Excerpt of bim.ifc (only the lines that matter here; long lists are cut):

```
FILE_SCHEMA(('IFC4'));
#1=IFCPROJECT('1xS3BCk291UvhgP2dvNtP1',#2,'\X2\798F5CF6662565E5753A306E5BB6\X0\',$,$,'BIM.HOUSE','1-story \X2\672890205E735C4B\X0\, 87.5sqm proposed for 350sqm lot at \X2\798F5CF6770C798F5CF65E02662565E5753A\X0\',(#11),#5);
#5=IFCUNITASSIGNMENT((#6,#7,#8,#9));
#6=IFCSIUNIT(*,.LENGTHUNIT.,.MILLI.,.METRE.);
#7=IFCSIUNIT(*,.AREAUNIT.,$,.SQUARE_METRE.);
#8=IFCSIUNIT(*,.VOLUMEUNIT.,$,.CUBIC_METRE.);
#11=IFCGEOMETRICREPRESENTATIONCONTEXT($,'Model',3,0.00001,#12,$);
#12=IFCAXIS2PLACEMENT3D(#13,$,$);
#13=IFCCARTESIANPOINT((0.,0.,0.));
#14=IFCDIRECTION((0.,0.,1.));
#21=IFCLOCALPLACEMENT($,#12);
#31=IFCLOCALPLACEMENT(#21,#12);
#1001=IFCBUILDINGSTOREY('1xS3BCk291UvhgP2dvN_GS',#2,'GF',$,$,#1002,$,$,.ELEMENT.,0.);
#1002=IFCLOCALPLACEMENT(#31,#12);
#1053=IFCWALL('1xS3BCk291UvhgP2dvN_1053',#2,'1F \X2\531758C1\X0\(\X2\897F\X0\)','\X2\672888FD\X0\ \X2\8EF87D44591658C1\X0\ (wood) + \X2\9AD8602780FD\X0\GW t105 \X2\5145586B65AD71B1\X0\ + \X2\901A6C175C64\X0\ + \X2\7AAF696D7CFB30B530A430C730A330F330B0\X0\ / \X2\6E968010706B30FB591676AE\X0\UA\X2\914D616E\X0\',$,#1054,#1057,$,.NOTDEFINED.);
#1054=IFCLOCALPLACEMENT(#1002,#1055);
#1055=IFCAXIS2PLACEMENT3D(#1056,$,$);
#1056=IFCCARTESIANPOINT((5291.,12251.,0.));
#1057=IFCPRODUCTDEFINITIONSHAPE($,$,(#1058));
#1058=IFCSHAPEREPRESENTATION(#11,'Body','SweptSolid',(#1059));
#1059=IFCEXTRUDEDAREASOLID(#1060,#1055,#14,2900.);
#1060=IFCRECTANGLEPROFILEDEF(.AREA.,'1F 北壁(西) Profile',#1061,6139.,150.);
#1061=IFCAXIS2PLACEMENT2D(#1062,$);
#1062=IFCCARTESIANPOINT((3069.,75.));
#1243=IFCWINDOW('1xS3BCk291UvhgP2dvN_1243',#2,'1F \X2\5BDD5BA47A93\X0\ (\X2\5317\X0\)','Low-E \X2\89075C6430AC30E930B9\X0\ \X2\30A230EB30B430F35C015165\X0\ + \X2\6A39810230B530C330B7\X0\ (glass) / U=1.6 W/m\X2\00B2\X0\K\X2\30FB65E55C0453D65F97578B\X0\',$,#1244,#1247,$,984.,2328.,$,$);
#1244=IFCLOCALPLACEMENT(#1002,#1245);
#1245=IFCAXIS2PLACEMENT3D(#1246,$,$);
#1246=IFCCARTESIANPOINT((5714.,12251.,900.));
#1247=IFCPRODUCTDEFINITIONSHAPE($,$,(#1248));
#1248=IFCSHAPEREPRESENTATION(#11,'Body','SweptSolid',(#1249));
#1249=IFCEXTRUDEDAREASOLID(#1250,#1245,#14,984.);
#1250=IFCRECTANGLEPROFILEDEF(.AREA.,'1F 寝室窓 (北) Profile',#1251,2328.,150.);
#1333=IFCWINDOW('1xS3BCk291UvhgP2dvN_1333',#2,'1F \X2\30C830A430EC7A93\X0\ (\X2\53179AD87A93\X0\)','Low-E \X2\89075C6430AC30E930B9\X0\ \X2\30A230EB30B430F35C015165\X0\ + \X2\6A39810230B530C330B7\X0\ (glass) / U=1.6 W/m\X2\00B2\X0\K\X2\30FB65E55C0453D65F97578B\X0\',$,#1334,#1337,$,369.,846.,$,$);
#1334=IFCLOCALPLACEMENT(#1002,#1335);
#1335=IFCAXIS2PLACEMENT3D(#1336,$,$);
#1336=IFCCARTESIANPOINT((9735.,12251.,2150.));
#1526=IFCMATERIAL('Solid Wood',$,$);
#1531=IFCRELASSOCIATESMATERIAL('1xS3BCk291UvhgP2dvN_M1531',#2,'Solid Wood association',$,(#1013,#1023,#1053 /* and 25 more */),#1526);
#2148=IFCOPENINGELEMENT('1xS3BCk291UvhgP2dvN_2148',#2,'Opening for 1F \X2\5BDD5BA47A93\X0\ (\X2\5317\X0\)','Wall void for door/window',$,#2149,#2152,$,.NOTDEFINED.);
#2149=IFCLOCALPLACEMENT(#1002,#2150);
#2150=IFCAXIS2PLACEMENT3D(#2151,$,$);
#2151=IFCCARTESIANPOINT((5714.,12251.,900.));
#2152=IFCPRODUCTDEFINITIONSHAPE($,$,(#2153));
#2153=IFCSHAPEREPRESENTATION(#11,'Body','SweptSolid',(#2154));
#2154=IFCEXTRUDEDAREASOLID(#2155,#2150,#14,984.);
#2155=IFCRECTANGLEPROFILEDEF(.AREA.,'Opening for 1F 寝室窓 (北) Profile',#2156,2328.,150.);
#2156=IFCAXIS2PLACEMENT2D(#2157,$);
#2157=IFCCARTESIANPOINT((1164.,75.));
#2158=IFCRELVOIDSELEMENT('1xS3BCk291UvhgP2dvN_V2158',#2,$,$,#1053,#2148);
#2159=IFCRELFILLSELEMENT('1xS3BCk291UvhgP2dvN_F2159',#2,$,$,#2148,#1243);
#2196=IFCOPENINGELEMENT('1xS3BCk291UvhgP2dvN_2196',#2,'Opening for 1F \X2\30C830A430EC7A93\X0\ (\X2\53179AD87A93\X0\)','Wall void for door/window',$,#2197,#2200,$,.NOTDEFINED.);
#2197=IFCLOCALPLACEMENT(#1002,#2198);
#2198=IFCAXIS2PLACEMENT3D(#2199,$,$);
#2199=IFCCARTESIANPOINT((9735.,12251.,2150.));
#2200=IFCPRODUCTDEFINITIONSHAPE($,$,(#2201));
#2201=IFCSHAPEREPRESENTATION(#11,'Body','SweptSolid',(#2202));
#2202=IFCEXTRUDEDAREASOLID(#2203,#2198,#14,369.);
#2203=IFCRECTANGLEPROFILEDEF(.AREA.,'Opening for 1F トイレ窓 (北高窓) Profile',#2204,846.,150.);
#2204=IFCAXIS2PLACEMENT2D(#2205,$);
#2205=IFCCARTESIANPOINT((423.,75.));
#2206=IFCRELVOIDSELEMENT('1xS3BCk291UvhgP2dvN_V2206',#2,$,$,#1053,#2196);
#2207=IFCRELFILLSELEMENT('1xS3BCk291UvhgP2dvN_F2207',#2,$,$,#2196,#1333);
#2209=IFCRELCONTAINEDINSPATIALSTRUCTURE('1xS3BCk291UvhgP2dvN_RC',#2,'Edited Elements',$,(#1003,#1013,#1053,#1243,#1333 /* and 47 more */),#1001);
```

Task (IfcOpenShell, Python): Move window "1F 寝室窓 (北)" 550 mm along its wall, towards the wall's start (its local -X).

```python
import ifcopenshell
import ifcopenshell.api.geometry
import ifcopenshell.util.placement
import ifcopenshell.util.unit

model = ifcopenshell.open("bim.ifc")
unit_scale = ifcopenshell.util.unit.calculate_unit_scale(model)

window = model.by_guid("1xS3BCk291UvhgP2dvN_1243")
opening = window.FillsVoids[0].RelatingOpeningElement
wall = opening.VoidsElements[0].RelatingBuildingElement

wall_matrix = ifcopenshell.util.placement.get_local_placement(wall.ObjectPlacement)
shift = wall_matrix[:3, 0] * -0.55 / unit_scale
before = ifcopenshell.util.placement.get_local_placement(window.ObjectPlacement)[:3, 3].copy()

# The window is not placed relative to its opening, so move both.
for product in (opening, window):
    matrix = ifcopenshell.util.placement.get_local_placement(product.ObjectPlacement)
    matrix[:3, 3] += shift
    ifcopenshell.api.geometry.edit_object_placement(model, product=product, matrix=matrix, is_si=False)

after = ifcopenshell.util.placement.get_local_placement(window.ObjectPlacement)[:3, 3]
print("window moved by", (after - before).round(3) + 0.0)

model.write("bim-out.ifc")
```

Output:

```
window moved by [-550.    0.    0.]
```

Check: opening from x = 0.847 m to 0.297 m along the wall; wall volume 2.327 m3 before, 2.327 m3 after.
